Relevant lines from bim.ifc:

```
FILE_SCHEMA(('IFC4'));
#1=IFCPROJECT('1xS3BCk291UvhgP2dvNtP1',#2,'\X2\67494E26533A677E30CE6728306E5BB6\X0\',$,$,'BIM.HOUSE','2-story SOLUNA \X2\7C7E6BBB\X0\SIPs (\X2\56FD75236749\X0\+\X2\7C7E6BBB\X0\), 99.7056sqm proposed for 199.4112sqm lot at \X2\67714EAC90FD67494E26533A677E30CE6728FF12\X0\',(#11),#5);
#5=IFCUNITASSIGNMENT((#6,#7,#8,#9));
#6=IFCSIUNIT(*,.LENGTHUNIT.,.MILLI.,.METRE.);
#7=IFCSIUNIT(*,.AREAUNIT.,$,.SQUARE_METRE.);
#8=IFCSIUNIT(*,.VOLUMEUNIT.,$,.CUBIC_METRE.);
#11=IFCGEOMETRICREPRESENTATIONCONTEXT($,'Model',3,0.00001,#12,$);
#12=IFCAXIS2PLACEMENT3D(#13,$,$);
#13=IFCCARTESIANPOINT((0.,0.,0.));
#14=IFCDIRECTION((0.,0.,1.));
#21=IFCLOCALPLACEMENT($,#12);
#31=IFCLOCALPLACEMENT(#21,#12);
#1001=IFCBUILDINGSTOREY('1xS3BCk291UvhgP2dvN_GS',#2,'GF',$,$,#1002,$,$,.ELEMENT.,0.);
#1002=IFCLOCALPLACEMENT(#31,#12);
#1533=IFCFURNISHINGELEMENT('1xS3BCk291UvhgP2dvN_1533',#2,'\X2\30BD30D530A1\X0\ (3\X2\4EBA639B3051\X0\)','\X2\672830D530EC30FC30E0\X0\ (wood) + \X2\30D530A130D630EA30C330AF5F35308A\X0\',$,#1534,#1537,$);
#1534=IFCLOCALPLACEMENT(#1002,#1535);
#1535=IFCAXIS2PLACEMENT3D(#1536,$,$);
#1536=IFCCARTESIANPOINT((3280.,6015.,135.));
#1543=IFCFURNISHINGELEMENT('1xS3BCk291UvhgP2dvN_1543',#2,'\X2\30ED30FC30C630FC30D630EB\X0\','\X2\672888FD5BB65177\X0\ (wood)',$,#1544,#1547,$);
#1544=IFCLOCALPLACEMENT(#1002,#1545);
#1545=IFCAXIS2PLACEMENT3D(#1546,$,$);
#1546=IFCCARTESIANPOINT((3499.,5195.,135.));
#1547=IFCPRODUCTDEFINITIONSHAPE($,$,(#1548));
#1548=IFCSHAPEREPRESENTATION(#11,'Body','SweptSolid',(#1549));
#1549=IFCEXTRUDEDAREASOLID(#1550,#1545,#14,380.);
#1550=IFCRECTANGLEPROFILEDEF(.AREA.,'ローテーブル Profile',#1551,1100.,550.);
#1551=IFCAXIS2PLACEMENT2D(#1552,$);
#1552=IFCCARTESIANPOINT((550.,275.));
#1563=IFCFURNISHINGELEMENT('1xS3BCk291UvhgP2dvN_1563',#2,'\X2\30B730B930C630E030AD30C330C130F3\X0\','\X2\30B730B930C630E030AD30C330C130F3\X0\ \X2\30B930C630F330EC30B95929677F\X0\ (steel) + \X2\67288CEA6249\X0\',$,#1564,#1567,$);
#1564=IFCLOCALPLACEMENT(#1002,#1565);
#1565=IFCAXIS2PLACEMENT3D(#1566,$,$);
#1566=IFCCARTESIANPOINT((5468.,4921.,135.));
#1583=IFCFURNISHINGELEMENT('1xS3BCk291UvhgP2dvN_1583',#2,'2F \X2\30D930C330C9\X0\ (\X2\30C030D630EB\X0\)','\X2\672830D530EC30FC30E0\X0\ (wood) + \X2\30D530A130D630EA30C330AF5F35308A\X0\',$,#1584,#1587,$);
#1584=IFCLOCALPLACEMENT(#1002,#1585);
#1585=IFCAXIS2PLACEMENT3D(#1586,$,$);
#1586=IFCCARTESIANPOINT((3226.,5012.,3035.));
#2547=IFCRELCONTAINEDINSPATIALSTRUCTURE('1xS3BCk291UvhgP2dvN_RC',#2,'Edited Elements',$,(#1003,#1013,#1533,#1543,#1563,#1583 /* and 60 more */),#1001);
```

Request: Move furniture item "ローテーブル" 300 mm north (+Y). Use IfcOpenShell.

```python
import ifcopenshell
import ifcopenshell.api.geometry
import ifcopenshell.util.placement

model = ifcopenshell.open("bim.ifc")

item = model.by_guid("1xS3BCk291UvhgP2dvN_1543")
matrix = ifcopenshell.util.placement.get_local_placement(item.ObjectPlacement)
matrix[1, 3] += 300.0
ifcopenshell.api.geometry.edit_object_placement(model, product=item, matrix=matrix, is_si=False)

print(ifcopenshell.util.placement.get_local_placement(item.ObjectPlacement).round(3) + 0.0)

model.write("bim_v2.ifc")
```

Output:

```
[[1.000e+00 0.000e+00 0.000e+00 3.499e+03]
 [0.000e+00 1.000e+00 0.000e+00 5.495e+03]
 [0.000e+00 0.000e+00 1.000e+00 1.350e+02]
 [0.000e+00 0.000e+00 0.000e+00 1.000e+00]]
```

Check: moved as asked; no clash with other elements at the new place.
